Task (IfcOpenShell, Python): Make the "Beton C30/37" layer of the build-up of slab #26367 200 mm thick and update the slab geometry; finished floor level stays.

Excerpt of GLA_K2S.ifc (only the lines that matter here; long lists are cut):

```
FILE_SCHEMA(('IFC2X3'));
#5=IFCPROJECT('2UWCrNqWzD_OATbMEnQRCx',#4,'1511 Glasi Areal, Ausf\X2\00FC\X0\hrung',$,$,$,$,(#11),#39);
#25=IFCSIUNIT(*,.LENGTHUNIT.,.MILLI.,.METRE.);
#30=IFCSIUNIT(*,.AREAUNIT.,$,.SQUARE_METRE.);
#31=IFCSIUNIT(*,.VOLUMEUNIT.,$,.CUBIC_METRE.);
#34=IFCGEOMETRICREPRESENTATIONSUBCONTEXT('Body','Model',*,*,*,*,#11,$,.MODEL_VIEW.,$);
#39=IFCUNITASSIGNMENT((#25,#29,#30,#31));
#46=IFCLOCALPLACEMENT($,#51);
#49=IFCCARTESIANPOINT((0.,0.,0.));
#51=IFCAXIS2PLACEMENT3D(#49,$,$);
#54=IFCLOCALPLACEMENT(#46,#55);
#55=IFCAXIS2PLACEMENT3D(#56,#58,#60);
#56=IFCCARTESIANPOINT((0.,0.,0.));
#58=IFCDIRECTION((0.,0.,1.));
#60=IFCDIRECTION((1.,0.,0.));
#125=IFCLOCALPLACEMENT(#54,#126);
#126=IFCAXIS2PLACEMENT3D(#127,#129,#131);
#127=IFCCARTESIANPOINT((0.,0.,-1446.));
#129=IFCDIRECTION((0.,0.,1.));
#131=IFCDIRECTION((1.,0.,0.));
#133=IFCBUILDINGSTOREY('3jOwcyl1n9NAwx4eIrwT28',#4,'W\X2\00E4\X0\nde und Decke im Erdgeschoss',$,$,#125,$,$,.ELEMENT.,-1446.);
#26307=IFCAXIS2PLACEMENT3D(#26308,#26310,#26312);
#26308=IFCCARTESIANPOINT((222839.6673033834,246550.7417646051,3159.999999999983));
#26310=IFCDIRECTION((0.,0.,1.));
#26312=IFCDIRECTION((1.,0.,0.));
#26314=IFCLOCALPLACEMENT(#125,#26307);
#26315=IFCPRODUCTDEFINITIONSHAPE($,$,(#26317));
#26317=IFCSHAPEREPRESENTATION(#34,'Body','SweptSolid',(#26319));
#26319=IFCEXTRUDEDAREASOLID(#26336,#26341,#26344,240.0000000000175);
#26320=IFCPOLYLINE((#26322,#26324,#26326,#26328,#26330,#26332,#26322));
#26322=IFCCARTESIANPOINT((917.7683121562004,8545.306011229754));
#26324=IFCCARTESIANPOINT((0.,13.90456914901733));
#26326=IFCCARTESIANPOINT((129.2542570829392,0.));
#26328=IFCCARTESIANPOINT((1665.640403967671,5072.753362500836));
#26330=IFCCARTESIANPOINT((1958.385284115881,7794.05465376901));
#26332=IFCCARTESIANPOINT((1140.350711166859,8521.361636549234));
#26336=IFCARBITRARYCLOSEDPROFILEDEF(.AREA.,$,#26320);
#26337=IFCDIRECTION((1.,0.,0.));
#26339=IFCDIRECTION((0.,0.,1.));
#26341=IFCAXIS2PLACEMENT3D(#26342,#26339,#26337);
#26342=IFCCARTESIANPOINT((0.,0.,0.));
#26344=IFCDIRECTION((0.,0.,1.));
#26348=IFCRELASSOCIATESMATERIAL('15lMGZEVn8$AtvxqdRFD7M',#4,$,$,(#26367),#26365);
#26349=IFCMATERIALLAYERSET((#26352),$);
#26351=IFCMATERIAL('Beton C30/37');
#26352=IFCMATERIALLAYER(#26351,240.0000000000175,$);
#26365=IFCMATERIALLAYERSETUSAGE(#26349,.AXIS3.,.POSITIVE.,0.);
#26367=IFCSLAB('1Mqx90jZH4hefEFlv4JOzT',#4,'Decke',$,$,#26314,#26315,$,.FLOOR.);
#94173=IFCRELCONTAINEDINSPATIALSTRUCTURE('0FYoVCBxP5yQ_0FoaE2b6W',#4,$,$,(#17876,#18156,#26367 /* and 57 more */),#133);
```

```python
import ifcopenshell
import ifcopenshell.util.element
import ifcopenshell.util.representation

model = ifcopenshell.open("GLA_K2S.ifc")

layer_set = model.by_id(26349)
layer = next(l for l in layer_set.MaterialLayers if l.Material and l.Material.Name == "Beton C30/37")
change = 200.0 - layer.LayerThickness
layer.LayerThickness += change

# Geometry does not follow the layer set by itself.
slabs = [e for e in ifcopenshell.util.element.get_elements_by_material(model, layer_set) if e.is_a("IfcSlab")]
for slab in sorted(slabs, key=lambda e: e.id()):
    body = ifcopenshell.util.representation.get_representation(slab, "Model", "Body")
    solid = body.Items[0]
    old_depth = solid.Depth
    solid.Depth += change
    # Extruded upwards: lower the start of the extrusion so the top stays.
    x, y, z = solid.Position.Location.Coordinates
    solid.Position.Location = model.createIfcCartesianPoint((x, y, z - change))
    print(slab.id(), f"{old_depth:g} -> {solid.Depth:g}")

# The layers are counted up from the underside, which has moved.
for usage in {ifcopenshell.util.element.get_material(slab) for slab in slabs}:
    usage.OffsetFromReferenceLine -= change

model.write("GLA_K2S-out.ifc")
```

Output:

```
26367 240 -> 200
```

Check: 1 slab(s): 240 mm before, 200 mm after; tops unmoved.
